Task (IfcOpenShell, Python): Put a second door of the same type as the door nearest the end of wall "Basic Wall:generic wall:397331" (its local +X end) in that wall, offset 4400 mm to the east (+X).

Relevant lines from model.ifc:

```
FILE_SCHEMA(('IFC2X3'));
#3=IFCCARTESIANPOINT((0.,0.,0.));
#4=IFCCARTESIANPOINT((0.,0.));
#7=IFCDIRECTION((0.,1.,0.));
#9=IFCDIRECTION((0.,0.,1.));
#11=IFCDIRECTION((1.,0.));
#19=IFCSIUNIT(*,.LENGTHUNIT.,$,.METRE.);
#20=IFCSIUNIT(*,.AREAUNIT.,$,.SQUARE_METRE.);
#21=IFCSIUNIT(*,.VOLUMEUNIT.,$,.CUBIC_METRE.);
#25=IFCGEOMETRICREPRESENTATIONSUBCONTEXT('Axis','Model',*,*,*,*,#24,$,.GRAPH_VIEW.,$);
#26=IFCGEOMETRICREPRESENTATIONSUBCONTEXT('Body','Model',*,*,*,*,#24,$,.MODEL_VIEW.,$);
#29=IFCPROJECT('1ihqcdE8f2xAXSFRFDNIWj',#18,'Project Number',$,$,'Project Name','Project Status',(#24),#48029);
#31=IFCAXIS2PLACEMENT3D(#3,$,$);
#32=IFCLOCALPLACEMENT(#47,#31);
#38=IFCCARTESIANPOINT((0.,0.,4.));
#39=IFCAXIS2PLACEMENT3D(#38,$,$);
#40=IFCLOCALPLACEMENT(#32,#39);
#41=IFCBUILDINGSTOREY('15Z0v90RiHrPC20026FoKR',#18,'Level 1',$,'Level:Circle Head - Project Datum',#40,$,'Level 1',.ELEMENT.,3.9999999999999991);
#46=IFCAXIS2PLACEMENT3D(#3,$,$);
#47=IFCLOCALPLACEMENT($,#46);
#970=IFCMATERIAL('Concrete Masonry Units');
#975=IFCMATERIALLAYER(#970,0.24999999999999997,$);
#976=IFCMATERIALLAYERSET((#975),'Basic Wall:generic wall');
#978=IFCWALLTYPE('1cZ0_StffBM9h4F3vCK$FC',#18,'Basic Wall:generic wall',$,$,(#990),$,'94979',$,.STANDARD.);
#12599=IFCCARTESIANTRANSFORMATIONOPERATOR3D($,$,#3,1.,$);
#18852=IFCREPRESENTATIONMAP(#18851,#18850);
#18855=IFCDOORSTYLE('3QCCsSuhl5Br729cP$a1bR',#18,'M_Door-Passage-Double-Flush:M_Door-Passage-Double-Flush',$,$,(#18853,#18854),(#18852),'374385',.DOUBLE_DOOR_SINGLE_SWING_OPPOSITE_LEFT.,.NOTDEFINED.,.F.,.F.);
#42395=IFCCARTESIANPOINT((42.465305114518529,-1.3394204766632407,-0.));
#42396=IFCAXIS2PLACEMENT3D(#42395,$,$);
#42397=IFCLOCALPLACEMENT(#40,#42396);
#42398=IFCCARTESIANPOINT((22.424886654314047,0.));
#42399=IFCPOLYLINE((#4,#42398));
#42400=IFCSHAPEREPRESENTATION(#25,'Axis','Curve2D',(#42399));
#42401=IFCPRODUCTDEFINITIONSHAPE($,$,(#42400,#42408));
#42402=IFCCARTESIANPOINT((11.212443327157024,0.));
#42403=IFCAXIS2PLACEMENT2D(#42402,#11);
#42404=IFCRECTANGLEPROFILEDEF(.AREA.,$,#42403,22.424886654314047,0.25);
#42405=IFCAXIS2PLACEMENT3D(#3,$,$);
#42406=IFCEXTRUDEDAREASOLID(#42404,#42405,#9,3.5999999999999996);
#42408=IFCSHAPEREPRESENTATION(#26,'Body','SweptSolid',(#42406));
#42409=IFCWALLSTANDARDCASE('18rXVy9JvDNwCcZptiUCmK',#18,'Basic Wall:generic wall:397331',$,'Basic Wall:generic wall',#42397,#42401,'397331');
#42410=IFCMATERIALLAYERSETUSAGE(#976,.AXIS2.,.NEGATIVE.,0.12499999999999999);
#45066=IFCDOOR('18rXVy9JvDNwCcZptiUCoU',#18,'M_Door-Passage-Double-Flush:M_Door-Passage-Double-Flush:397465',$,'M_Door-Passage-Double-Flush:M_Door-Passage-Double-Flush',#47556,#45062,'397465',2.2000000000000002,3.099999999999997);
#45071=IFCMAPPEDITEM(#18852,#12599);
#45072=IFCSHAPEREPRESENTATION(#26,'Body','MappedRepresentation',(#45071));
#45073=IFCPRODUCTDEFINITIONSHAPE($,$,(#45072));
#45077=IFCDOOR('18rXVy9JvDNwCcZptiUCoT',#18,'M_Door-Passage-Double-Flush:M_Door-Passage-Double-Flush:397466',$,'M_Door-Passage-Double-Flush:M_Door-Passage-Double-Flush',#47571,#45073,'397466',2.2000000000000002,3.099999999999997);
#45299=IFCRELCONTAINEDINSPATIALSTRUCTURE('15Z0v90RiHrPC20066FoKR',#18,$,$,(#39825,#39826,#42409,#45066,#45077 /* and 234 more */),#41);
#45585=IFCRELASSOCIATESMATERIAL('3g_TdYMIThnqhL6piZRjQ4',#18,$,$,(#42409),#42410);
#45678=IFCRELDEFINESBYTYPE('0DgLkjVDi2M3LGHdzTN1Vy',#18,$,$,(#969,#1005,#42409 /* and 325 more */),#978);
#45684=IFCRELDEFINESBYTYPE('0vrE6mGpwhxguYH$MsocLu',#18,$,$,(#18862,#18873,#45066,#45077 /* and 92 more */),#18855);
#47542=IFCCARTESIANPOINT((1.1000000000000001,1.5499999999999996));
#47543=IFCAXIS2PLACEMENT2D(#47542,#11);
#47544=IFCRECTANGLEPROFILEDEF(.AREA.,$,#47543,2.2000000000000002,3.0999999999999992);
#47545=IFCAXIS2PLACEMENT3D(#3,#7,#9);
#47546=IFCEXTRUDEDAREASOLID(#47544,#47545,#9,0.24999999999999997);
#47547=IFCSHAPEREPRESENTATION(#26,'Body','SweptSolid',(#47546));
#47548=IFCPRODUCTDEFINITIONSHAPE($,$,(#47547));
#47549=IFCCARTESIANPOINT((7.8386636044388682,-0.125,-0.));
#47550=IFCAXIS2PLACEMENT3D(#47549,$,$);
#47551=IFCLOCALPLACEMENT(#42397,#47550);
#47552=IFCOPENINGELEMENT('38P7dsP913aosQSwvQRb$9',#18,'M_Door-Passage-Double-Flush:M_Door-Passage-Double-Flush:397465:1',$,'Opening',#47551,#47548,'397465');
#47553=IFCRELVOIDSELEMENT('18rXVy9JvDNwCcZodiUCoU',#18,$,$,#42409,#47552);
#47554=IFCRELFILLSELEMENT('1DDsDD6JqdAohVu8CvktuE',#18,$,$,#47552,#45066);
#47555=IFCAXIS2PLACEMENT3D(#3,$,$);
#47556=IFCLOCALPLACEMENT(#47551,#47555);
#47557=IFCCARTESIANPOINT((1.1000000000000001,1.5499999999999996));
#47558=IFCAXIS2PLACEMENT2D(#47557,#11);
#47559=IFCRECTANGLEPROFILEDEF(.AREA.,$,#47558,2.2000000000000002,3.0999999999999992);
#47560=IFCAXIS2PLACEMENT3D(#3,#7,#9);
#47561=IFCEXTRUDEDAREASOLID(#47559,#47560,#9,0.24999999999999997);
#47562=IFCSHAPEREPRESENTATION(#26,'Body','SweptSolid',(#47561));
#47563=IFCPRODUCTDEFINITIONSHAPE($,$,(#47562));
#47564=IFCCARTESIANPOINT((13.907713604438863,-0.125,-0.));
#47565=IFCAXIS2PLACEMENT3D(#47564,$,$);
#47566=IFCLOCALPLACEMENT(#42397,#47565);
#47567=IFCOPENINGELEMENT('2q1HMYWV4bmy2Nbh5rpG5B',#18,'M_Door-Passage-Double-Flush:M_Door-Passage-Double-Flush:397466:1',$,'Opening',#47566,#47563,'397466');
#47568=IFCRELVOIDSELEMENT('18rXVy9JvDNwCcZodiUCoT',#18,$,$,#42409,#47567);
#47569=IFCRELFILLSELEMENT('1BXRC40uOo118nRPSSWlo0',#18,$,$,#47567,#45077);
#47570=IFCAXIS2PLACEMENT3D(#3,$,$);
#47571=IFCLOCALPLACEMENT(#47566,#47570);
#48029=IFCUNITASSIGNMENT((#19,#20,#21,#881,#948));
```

```python
import ifcopenshell
import ifcopenshell.api.feature
import ifcopenshell.api.geometry
import ifcopenshell.api.root
import ifcopenshell.geom
import ifcopenshell.util.element
import ifcopenshell.util.placement
import ifcopenshell.util.shape

model = ifcopenshell.open("model.ifc")
settings = ifcopenshell.geom.settings()


def volume(element):
    """Net volume in cubic metres, openings subtracted."""
    shape = ifcopenshell.geom.create_shape(settings, element)
    return ifcopenshell.util.shape.get_volume(shape.geometry)


def reuse_history(source, copy):
    """copy_class also copies each property set's owner history, people and application; keep the originals."""
    for rel in copy.IsDefinedBy:
        if rel.is_a("IfcRelDefinesByProperties") and (history := rel.RelatingPropertyDefinition.OwnerHistory):
            rel.RelatingPropertyDefinition.OwnerHistory = source.OwnerHistory
            ifcopenshell.util.element.remove_deep2(model, history)


door = model.by_guid("18rXVy9JvDNwCcZptiUCoT")
opening = door.FillsVoids[0].RelatingOpeningElement
wall = opening.VoidsElements[0].RelatingBuildingElement
before = volume(wall)
shift = ifcopenshell.util.placement.get_local_placement(wall.ObjectPlacement)[:3, 0] * 4.4

# copy_class copies the void relationship, type, container and properties, but no geometry.
new_opening = ifcopenshell.api.root.copy_class(model, product=opening)
new_opening.Representation = ifcopenshell.util.element.copy_deep(
    model, opening.Representation, exclude=["IfcGeometricRepresentationContext", "IfcRepresentationMap"]
)
new_opening.Name = "M_Door-Passage-Double-Flush:M_Door-Passage-Double-Flush"
new_opening.Tag = None
new_door = ifcopenshell.api.root.copy_class(model, product=door)
new_door.Representation = ifcopenshell.util.element.copy_deep(
    model, door.Representation, exclude=["IfcGeometricRepresentationContext", "IfcRepresentationMap"]
)
new_door.Name = "M_Door-Passage-Double-Flush:M_Door-Passage-Double-Flush"
new_door.Tag = None
reuse_history(door, new_door)
fills = ifcopenshell.api.feature.add_filling(model, opening=new_opening, element=new_door)
fills.OwnerHistory = new_door.OwnerHistory  # required in IFC2X3

for old, new in ((opening, new_opening), (door, new_door)):
    matrix = ifcopenshell.util.placement.get_local_placement(old.ObjectPlacement)
    matrix[:3, 3] += shift
    ifcopenshell.api.geometry.edit_object_placement(model, product=new, matrix=matrix, is_si=False)

after = volume(wall)

print(f"wall volume {before:.3f} -> {after:.3f} m3")

model.write("model_rev.ifc")
```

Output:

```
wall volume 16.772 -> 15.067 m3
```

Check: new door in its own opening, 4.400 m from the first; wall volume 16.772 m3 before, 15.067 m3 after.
